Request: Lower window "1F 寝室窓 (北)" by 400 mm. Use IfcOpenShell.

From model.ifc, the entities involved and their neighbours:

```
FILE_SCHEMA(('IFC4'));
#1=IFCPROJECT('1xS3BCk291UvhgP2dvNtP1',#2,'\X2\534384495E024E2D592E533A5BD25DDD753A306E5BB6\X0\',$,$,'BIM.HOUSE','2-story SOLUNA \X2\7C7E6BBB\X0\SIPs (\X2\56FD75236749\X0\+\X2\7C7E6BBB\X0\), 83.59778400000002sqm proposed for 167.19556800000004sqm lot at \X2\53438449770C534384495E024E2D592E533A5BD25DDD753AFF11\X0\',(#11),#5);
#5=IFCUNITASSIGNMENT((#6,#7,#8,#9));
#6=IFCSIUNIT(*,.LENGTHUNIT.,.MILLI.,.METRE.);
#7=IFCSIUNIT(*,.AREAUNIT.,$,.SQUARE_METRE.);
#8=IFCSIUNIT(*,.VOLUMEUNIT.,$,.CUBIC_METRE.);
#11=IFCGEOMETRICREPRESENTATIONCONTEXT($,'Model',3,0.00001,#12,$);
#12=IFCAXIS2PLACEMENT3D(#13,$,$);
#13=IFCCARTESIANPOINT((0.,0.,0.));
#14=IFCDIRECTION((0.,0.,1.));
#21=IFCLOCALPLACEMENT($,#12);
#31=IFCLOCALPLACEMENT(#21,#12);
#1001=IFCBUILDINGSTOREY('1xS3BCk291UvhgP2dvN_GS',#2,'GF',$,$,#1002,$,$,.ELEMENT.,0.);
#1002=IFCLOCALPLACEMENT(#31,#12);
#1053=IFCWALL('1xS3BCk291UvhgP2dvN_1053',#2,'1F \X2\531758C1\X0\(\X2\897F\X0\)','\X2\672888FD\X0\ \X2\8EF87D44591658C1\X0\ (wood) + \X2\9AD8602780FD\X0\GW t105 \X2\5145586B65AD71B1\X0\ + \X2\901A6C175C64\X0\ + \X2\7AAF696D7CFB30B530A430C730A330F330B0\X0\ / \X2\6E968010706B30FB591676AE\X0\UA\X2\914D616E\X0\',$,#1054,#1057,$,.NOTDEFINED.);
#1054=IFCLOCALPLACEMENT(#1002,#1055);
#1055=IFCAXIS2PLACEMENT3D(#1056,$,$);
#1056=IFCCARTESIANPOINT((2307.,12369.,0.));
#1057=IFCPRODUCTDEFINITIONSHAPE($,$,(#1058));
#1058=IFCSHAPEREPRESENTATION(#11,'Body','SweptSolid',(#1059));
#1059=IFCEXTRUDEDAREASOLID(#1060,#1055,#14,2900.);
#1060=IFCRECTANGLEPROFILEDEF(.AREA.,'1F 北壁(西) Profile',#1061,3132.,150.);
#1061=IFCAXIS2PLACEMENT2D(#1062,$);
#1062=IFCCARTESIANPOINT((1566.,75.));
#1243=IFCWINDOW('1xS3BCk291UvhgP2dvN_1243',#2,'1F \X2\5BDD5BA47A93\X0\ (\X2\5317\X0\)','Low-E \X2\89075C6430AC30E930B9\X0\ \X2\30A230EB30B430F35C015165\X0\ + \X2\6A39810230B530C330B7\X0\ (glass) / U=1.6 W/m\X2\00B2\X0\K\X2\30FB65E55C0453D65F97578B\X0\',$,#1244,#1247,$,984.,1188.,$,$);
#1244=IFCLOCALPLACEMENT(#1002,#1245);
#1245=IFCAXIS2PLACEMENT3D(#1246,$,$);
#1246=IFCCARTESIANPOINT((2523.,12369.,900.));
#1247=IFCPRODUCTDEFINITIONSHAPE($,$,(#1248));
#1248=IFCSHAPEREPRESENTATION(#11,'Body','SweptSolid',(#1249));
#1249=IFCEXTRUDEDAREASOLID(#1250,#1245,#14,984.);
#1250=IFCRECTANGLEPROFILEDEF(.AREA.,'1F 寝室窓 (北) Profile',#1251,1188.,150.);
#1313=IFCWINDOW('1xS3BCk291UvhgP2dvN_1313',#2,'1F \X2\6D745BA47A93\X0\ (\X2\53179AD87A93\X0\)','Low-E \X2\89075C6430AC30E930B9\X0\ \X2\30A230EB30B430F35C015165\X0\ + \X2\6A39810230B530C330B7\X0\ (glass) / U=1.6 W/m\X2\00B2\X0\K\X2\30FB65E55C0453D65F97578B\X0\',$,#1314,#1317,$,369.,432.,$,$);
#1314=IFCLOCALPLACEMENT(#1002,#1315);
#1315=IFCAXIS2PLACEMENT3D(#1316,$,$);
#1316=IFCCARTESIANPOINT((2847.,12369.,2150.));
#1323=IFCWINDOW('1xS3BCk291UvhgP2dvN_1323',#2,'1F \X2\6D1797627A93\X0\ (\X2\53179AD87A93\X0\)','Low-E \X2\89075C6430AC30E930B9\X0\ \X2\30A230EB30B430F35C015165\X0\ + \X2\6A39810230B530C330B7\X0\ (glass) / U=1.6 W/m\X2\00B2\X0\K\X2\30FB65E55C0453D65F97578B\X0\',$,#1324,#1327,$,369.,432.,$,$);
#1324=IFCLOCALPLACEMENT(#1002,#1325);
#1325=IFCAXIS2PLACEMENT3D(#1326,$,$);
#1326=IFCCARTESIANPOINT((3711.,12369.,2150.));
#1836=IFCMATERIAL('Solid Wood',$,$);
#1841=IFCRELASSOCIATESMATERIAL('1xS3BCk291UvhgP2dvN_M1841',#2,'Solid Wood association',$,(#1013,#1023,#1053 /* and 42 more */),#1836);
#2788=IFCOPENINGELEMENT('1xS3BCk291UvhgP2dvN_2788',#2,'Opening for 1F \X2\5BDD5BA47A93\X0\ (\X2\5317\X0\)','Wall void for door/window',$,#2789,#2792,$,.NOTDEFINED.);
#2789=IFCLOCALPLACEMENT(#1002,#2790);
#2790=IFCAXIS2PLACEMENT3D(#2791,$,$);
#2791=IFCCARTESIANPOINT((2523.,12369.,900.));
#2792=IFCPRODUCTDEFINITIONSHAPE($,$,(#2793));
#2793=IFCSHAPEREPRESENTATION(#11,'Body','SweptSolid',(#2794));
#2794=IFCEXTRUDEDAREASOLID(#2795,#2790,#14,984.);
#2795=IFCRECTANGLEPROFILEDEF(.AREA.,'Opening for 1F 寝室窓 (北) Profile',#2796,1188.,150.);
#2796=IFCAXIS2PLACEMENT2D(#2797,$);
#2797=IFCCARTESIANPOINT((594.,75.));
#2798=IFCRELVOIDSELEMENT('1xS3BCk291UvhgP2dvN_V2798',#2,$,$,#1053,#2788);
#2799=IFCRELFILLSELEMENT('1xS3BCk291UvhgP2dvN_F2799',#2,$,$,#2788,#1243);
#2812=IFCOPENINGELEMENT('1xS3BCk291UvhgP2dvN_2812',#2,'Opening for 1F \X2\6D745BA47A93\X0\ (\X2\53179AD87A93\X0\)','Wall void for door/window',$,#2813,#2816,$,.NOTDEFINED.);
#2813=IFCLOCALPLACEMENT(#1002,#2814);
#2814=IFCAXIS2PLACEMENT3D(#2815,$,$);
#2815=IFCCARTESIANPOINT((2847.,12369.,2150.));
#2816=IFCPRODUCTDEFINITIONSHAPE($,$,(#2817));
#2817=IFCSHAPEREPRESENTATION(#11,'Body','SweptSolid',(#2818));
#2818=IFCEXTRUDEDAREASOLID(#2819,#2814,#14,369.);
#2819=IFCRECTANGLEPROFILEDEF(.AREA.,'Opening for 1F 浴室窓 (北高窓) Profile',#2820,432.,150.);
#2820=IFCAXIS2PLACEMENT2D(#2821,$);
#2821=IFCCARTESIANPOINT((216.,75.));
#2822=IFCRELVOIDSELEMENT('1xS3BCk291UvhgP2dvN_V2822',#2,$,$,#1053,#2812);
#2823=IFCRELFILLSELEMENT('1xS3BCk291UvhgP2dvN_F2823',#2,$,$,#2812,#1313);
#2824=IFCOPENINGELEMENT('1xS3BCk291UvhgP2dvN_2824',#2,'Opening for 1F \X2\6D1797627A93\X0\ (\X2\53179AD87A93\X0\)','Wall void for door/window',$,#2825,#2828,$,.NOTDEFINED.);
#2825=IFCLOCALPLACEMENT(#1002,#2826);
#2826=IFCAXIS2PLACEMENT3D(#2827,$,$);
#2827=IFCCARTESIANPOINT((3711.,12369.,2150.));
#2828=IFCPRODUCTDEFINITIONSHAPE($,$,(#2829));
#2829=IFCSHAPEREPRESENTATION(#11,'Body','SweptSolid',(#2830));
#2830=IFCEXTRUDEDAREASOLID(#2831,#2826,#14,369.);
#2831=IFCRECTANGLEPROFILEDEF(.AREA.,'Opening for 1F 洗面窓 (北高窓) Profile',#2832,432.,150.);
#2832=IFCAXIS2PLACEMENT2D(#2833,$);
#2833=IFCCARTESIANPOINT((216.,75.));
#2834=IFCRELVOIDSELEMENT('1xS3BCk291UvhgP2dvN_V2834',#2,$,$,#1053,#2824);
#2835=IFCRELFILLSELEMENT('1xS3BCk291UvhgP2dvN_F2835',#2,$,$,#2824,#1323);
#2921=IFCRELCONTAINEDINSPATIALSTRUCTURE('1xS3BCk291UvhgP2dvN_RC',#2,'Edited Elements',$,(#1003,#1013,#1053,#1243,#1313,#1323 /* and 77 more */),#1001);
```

```python
import numpy as np
import ifcopenshell
import ifcopenshell.api.geometry
import ifcopenshell.util.placement
import ifcopenshell.util.unit

model = ifcopenshell.open("model.ifc")
unit_scale = ifcopenshell.util.unit.calculate_unit_scale(model)

window = model.by_guid("1xS3BCk291UvhgP2dvN_1243")
opening = window.FillsVoids[0].RelatingOpeningElement
dz = -0.4 / unit_scale

shift = np.array([0.0, 0.0, dz])
# The window is not placed relative to its opening, so move both.
for product in (opening, window):
    matrix = ifcopenshell.util.placement.get_local_placement(product.ObjectPlacement)
    matrix[:3, 3] += shift
    ifcopenshell.api.geometry.edit_object_placement(model, product=product, matrix=matrix, is_si=False)

print(f"moved by {dz * unit_scale:+.3f} m")

model.write("model_edited.ifc")
```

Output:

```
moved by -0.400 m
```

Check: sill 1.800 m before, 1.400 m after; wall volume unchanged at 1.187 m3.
